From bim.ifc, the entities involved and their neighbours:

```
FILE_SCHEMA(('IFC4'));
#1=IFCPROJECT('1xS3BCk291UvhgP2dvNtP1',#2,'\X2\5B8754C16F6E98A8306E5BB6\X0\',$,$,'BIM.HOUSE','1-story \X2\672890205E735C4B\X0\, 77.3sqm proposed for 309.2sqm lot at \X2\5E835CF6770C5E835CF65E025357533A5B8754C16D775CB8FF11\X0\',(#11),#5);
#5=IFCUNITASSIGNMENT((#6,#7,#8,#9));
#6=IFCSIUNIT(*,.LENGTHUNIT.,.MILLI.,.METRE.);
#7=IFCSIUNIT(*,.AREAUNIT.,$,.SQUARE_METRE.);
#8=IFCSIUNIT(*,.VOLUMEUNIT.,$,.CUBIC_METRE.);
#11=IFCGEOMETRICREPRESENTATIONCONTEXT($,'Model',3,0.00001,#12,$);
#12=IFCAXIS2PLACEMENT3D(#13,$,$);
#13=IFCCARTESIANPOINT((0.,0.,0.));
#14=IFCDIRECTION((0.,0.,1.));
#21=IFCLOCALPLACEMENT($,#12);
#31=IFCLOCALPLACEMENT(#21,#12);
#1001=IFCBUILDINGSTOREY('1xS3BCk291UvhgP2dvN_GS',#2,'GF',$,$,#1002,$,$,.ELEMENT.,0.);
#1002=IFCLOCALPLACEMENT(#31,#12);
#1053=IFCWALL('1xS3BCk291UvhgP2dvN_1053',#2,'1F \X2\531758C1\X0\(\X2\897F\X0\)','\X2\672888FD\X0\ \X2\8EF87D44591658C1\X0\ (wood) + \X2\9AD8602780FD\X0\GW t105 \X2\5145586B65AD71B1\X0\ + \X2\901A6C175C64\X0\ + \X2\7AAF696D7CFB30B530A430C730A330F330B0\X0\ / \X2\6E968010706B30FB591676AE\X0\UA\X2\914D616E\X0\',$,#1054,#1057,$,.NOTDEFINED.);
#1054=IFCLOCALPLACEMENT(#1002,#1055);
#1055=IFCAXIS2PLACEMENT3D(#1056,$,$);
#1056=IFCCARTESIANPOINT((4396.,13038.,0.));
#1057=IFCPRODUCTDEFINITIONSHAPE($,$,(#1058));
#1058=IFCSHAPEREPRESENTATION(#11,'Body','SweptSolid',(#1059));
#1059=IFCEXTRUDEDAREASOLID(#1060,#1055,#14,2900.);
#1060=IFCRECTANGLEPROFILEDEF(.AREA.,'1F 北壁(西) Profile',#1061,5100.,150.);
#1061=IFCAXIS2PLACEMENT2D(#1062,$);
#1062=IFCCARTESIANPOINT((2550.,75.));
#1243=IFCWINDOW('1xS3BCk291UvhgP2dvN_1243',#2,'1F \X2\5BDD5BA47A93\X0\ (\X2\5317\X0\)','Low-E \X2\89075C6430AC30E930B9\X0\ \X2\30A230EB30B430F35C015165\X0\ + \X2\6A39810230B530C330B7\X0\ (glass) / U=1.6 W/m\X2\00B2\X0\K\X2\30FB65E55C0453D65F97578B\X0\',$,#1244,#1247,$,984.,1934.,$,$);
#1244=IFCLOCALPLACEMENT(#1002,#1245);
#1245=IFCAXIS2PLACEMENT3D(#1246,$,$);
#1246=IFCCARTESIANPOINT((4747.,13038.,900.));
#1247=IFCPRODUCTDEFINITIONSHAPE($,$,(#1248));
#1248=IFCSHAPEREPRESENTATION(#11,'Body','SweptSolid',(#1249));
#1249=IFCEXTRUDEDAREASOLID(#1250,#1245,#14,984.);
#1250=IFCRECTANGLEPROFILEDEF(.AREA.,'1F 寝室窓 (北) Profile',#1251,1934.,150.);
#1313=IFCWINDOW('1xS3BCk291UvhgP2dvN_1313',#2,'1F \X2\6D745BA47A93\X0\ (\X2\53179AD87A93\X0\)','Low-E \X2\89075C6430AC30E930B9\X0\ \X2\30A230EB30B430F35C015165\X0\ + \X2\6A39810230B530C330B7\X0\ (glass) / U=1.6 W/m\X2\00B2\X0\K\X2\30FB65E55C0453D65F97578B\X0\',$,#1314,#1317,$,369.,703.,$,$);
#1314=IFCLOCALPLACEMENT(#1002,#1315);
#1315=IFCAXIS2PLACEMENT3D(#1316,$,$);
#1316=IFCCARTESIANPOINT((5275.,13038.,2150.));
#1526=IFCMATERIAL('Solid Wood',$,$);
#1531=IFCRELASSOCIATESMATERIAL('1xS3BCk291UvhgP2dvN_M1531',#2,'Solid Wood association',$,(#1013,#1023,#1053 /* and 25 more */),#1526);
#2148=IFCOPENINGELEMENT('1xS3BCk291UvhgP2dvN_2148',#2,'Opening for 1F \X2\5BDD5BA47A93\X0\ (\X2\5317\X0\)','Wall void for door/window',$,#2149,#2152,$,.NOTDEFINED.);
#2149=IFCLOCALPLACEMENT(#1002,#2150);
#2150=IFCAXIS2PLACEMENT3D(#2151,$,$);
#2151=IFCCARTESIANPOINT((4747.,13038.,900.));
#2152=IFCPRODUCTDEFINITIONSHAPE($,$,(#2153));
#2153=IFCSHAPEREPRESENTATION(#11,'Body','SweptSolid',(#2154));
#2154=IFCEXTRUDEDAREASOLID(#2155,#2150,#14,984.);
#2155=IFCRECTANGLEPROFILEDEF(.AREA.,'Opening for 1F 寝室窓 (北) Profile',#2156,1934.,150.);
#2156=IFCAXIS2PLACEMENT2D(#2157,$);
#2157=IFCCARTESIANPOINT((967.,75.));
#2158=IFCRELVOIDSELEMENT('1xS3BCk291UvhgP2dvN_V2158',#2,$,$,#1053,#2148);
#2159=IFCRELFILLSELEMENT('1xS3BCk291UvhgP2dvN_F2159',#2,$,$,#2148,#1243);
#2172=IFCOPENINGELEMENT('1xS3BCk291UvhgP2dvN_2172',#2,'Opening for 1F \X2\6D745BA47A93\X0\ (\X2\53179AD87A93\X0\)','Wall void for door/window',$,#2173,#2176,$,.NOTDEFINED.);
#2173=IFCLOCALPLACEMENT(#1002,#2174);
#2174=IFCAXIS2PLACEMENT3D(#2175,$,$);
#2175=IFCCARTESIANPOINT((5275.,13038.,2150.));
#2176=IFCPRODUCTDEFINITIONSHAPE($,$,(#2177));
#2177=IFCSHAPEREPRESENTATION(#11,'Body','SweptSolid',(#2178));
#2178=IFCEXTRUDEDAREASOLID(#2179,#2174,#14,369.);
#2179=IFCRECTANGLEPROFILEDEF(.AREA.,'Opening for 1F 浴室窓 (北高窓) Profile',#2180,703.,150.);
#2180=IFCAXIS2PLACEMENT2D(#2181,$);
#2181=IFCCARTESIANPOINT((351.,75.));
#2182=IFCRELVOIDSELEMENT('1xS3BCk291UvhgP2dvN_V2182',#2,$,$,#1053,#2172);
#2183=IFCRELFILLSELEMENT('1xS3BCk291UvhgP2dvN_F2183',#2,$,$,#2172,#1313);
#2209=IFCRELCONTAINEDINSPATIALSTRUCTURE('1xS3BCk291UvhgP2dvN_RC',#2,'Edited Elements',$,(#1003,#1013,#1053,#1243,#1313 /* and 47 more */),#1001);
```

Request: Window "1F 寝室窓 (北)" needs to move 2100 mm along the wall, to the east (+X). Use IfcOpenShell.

```python
import ifcopenshell
import ifcopenshell.api.geometry
import ifcopenshell.util.placement
import ifcopenshell.util.unit

model = ifcopenshell.open("bim.ifc")
unit_scale = ifcopenshell.util.unit.calculate_unit_scale(model)

window = model.by_guid("1xS3BCk291UvhgP2dvN_1243")
opening = window.FillsVoids[0].RelatingOpeningElement
wall = opening.VoidsElements[0].RelatingBuildingElement

wall_matrix = ifcopenshell.util.placement.get_local_placement(wall.ObjectPlacement)
shift = wall_matrix[:3, 0] * 2.1 / unit_scale
before = ifcopenshell.util.placement.get_local_placement(window.ObjectPlacement)[:3, 3].copy()

# The window is not placed relative to its opening, so move both.
for product in (opening, window):
    matrix = ifcopenshell.util.placement.get_local_placement(product.ObjectPlacement)
    matrix[:3, 3] += shift
    ifcopenshell.api.geometry.edit_object_placement(model, product=product, matrix=matrix, is_si=False)

after = ifcopenshell.util.placement.get_local_placement(window.ObjectPlacement)[:3, 3]
print("window moved by", (after - before).round(3) + 0.0)

model.write("bim-out.ifc")
```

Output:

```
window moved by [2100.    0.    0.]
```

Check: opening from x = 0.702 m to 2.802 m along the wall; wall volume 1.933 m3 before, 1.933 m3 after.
